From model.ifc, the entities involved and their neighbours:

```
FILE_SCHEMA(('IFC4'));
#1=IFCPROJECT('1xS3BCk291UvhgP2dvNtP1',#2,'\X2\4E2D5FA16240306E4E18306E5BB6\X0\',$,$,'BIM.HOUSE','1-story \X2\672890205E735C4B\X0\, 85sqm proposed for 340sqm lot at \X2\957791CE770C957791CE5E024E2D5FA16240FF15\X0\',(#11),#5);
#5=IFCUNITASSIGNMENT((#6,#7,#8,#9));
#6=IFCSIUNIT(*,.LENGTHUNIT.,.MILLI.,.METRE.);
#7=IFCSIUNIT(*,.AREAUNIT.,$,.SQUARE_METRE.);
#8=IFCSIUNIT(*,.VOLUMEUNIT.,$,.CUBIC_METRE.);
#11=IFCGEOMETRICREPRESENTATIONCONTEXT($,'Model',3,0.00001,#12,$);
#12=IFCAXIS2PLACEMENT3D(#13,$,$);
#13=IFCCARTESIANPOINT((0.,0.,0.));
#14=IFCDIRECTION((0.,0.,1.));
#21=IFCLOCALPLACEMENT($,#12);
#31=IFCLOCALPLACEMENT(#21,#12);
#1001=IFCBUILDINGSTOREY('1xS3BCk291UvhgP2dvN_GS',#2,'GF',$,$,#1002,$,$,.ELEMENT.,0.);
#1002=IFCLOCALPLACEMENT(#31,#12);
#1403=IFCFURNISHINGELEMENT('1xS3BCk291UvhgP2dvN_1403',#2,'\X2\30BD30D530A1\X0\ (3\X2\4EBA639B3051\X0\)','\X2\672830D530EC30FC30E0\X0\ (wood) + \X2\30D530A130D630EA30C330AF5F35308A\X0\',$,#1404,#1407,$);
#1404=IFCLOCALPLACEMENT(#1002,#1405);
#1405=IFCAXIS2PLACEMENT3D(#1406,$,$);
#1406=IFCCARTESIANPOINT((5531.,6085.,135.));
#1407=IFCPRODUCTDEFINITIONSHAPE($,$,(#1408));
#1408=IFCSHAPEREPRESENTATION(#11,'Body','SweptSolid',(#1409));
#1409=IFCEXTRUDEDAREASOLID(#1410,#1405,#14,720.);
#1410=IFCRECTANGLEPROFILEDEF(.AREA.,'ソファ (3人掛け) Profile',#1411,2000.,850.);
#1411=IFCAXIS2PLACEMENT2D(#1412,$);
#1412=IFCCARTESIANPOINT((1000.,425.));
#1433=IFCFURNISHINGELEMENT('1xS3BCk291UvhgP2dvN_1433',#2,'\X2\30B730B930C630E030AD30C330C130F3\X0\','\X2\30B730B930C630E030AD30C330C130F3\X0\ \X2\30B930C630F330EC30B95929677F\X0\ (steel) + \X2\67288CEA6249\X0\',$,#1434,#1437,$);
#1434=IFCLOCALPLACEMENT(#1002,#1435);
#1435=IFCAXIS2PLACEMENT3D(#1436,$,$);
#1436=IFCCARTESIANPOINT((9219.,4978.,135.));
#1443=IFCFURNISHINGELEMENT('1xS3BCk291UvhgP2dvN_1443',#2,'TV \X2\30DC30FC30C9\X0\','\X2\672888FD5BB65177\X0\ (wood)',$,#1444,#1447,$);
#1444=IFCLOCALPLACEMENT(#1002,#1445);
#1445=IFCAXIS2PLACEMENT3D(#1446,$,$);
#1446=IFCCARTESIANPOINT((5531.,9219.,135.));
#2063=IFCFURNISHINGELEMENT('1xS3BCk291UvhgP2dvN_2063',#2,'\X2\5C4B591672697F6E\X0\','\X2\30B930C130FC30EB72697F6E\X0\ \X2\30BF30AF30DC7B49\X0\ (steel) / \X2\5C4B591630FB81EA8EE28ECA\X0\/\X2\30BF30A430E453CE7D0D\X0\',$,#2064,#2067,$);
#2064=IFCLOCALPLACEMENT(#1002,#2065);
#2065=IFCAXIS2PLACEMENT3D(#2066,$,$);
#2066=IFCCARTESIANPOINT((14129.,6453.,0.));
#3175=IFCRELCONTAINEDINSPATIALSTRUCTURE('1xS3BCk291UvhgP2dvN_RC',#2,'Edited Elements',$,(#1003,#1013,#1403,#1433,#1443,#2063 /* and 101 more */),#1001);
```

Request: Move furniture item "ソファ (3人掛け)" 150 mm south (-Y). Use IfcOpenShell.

```python
import ifcopenshell
import ifcopenshell.api.geometry
import ifcopenshell.util.placement

model = ifcopenshell.open("model.ifc")

item = model.by_guid("1xS3BCk291UvhgP2dvN_1403")
matrix = ifcopenshell.util.placement.get_local_placement(item.ObjectPlacement)
matrix[1, 3] -= 150.0
ifcopenshell.api.geometry.edit_object_placement(model, product=item, matrix=matrix, is_si=False)

print(ifcopenshell.util.placement.get_local_placement(item.ObjectPlacement).round(3) + 0.0)

model.write("model_v2.ifc")
```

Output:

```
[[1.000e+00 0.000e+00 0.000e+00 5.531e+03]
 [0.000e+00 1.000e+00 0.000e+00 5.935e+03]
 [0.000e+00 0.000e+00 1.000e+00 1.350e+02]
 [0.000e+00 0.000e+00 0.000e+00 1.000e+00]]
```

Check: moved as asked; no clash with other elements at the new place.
